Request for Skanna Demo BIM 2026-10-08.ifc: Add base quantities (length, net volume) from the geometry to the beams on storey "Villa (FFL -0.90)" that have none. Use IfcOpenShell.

First a look at what the model holds.

```python
import ifcopenshell
import ifcopenshell.util.element
import ifcopenshell.util.unit

model = ifcopenshell.open("Skanna Demo BIM 2026-10-08.ifc")
print(model.schema)
for unit_type in ("LENGTHUNIT", "AREAUNIT", "VOLUMEUNIT"):
    print(unit_type, ifcopenshell.util.unit.calculate_unit_scale(model, unit_type))
storey = next(s for s in model.by_type("IfcBuildingStorey") if s.Name == "Villa (FFL -0.90)")
beams = [e for e in ifcopenshell.util.element.get_decomposition(storey) if e.is_a("IfcBeam")]
for e in sorted(beams, key=lambda e: e.id()):
    print(e.id(), e.is_a(), e.Name, list(ifcopenshell.util.element.get_psets(e, qtos_only=True)), sep=" | ")
```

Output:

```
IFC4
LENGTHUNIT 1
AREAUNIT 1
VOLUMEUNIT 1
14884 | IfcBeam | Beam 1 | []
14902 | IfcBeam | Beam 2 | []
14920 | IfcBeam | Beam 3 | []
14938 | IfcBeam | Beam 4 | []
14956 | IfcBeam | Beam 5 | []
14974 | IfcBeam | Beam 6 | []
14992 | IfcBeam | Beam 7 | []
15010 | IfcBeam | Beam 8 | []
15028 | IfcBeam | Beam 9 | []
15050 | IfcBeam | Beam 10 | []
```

```python
import ifcopenshell
import ifcopenshell.api.pset
import ifcopenshell.geom
import ifcopenshell.util.element
import ifcopenshell.util.shape
import ifcopenshell.util.unit

model = ifcopenshell.open("Skanna Demo BIM 2026-10-08.ifc")
unit_scale = ifcopenshell.util.unit.calculate_unit_scale(model)
volume_scale = ifcopenshell.util.unit.calculate_unit_scale(model, "VOLUMEUNIT")
settings = ifcopenshell.geom.settings()

storey = next(s for s in model.by_type("IfcBuildingStorey") if s.Name == "Villa (FFL -0.90)")
beams = [e for e in ifcopenshell.util.element.get_decomposition(storey) if e.is_a("IfcBeam")]

for e in sorted(beams, key=lambda e: e.id()):
    if ifcopenshell.util.element.get_psets(e, qtos_only=True, should_inherit=False):
        continue
    # Geometry comes back in metres, in the element's own axes.
    shape = ifcopenshell.geom.create_shape(settings, e)
    values = {
        "Length": ifcopenshell.util.shape.get_max_xyz(shape.geometry) / unit_scale,
        "NetVolume": ifcopenshell.util.shape.get_volume(shape.geometry) / volume_scale,
    }
    qto = ifcopenshell.api.pset.add_qto(model, product=e, name="Qto_BeamBaseQuantities")
    ifcopenshell.api.pset.edit_qto(model, qto=qto, properties=values)
    print(e.id(), {k: round(v, 3) for k, v in values.items()})

model.write("Skanna Demo BIM 2026-10-08_rev.ifc")
```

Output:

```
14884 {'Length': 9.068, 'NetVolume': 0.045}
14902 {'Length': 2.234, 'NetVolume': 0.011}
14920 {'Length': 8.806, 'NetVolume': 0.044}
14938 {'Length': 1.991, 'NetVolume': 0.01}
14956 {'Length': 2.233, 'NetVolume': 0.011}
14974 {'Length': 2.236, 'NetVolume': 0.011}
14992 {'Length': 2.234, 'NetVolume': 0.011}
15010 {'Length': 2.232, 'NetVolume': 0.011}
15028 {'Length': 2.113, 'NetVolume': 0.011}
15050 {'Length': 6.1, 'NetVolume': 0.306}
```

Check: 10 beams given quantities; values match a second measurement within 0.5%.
